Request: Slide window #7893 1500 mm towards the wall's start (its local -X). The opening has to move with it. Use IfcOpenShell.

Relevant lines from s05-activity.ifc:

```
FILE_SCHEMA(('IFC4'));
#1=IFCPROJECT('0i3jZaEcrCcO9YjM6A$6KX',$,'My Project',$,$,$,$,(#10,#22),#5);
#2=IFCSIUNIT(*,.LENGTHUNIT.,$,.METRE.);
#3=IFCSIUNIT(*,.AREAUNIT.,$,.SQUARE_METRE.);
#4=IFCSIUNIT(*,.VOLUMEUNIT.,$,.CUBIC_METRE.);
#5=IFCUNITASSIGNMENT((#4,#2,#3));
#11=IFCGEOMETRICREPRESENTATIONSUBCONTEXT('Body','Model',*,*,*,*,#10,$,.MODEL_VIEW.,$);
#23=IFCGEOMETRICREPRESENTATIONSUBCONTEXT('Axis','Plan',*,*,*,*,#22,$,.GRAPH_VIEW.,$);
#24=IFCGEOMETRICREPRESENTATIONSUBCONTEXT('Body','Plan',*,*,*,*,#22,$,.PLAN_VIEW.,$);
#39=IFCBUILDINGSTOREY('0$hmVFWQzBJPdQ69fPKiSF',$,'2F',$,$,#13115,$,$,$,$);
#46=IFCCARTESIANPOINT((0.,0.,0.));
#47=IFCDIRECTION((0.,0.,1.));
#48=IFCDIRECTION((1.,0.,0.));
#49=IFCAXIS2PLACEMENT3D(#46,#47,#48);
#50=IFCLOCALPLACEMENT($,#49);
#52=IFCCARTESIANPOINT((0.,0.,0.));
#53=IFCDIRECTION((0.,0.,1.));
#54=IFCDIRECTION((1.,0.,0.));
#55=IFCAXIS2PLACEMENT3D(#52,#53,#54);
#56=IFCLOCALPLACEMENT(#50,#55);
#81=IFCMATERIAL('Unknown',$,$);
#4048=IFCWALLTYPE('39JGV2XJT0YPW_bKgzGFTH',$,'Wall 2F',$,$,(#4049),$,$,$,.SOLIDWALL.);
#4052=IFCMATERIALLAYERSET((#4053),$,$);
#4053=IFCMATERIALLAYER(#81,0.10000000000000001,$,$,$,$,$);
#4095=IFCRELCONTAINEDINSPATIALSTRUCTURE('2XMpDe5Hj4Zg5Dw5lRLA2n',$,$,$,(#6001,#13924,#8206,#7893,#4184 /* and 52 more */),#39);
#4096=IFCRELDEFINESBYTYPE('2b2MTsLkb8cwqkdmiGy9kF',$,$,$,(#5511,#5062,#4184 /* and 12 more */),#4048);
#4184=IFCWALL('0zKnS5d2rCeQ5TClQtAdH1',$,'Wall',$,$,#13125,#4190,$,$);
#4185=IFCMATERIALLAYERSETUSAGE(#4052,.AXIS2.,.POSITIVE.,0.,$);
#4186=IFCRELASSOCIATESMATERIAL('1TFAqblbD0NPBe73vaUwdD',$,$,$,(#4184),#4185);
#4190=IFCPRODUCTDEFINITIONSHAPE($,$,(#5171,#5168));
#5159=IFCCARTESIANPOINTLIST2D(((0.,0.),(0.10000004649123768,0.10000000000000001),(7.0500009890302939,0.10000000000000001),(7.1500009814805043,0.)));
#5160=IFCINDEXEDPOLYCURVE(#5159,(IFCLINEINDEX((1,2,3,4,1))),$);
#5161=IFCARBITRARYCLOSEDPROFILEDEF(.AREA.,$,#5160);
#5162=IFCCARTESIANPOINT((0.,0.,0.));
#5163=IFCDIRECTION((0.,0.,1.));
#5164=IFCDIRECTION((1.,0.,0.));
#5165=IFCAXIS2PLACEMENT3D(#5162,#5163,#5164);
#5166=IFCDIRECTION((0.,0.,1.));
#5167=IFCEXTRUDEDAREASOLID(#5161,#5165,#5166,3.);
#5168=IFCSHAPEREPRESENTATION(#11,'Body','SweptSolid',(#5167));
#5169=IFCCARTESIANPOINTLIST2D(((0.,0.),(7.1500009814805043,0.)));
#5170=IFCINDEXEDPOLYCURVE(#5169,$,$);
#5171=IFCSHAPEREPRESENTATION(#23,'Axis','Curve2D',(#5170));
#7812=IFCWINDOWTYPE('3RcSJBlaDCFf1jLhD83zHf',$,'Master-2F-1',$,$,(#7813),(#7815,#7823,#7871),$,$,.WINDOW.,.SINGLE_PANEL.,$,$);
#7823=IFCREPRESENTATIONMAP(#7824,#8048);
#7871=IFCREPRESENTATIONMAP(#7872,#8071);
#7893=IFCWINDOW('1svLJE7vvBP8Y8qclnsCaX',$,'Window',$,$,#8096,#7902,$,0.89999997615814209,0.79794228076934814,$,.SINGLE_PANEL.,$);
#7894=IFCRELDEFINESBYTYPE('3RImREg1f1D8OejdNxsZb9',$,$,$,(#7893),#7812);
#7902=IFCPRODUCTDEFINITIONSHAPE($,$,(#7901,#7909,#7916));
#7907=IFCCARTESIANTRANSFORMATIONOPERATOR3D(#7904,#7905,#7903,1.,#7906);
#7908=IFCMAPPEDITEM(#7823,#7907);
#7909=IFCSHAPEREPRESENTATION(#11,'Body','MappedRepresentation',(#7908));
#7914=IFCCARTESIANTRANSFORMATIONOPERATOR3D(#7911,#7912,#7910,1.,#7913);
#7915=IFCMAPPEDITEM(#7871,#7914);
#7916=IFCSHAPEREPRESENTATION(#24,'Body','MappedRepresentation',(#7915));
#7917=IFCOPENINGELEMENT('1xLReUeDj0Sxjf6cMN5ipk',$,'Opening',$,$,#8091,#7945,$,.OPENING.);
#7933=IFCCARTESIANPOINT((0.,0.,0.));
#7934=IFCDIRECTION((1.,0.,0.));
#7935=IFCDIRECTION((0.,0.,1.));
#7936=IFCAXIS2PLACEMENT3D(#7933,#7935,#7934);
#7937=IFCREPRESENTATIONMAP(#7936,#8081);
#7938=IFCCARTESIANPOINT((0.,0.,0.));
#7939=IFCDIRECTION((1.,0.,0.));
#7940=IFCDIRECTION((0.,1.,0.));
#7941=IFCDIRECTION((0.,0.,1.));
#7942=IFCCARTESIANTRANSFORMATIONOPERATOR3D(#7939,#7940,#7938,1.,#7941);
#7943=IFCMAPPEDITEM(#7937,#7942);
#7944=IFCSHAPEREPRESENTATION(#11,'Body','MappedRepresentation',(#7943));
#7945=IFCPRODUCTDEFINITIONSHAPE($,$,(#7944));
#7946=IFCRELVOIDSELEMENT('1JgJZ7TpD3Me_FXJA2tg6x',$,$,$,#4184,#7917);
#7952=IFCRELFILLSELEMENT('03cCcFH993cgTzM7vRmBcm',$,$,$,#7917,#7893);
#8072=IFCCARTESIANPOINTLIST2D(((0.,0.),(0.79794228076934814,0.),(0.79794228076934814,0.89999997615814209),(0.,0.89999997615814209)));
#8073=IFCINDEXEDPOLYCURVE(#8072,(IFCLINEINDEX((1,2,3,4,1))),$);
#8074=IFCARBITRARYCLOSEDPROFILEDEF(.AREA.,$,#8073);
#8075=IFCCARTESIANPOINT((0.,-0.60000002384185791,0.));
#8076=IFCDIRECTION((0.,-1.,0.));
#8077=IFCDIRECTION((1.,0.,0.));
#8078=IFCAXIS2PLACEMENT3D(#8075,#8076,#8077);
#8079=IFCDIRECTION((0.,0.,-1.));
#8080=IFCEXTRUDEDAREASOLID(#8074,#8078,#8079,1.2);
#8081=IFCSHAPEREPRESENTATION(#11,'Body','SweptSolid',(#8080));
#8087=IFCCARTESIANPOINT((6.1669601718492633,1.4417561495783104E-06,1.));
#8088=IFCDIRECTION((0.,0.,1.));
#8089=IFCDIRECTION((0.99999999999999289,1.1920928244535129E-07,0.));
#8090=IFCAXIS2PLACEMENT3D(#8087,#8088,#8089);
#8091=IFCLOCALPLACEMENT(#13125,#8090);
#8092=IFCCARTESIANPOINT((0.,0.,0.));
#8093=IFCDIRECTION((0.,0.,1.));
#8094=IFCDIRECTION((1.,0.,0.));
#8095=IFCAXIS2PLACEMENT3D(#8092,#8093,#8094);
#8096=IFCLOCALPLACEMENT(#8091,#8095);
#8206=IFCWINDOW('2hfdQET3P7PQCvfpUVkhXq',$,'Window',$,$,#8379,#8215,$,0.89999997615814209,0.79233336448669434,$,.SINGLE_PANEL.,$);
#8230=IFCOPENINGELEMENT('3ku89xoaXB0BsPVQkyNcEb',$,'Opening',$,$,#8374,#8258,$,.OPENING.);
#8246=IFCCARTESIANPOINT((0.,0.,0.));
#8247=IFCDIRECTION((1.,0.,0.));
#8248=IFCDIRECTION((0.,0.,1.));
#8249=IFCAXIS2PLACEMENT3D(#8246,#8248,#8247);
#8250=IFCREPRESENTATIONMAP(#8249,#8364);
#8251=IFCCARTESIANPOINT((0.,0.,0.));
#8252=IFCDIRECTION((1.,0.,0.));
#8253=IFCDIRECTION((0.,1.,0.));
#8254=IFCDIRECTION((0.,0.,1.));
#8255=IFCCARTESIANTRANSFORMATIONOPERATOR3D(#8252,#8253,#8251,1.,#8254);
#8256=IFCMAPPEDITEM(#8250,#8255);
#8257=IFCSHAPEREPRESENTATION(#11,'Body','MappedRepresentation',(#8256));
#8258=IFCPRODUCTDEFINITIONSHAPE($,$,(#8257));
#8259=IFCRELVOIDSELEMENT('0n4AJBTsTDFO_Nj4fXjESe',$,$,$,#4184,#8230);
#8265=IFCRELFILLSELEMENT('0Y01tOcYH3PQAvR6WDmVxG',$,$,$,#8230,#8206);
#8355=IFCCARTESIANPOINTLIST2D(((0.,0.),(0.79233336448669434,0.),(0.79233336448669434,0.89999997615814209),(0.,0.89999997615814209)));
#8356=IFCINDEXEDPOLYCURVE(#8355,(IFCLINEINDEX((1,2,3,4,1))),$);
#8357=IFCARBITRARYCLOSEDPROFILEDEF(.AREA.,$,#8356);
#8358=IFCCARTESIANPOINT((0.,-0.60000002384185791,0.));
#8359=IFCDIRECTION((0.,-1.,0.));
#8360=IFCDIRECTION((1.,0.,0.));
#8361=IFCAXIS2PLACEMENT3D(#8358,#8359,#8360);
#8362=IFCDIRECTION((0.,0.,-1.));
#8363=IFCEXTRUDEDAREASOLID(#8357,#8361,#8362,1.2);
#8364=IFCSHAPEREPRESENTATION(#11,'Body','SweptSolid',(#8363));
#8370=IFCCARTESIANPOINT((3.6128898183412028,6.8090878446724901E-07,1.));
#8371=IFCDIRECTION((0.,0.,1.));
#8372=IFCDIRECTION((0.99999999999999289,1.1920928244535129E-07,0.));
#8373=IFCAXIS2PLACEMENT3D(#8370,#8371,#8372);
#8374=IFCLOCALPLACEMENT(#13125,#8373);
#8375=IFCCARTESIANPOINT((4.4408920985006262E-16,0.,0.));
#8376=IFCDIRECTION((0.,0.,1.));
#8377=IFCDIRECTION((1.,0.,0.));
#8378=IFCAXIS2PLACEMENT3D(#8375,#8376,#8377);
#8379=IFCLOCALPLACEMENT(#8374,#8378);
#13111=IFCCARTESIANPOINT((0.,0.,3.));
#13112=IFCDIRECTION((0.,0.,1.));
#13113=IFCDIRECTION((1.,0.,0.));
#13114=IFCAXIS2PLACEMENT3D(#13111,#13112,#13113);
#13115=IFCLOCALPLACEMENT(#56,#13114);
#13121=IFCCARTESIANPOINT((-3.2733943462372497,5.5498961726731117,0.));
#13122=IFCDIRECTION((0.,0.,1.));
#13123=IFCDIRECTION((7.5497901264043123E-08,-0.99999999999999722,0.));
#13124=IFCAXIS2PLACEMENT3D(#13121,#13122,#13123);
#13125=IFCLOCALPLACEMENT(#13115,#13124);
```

```python
import ifcopenshell
import ifcopenshell.api.geometry
import ifcopenshell.util.placement
import ifcopenshell.util.unit

model = ifcopenshell.open("s05-activity.ifc")
unit_scale = ifcopenshell.util.unit.calculate_unit_scale(model)

window = model.by_guid("1svLJE7vvBP8Y8qclnsCaX")
opening = window.FillsVoids[0].RelatingOpeningElement
wall = opening.VoidsElements[0].RelatingBuildingElement

wall_matrix = ifcopenshell.util.placement.get_local_placement(wall.ObjectPlacement)
shift = wall_matrix[:3, 0] * -1.5 / unit_scale
before = ifcopenshell.util.placement.get_local_placement(window.ObjectPlacement)[:3, 3].copy()

# The window is placed relative to its opening, so it follows when the opening moves.
matrix = ifcopenshell.util.placement.get_local_placement(opening.ObjectPlacement)
matrix[:3, 3] += shift
ifcopenshell.api.geometry.edit_object_placement(
    model, product=opening, matrix=matrix, is_si=False, should_transform_children=True
)

after = ifcopenshell.util.placement.get_local_placement(window.ObjectPlacement)[:3, 3]
print("window moved by", (after - before).round(3) + 0.0)

model.write("s05-activity-out.ifc")
```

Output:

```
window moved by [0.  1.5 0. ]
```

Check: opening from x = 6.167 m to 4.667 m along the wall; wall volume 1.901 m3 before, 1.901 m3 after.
